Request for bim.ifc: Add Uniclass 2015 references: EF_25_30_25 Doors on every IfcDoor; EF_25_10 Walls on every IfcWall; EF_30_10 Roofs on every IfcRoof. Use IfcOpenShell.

First a look at what the model holds.

```python
import ifcopenshell

model = ifcopenshell.open("bim.ifc")
print(model.schema)
print("classifications:", [c.Name for c in model.by_type("IfcClassification")])
for ifc_class in ("IfcDoor", "IfcRoof", "IfcStair", "IfcWall", "IfcWindow"):
    print(ifc_class, len(model.by_type(ifc_class)))
```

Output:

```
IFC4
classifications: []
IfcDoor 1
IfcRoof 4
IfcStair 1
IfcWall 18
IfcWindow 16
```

```python
import ifcopenshell
import ifcopenshell.api.classification

model = ifcopenshell.open("bim.ifc")

system = ifcopenshell.api.classification.add_classification(model, classification="Uniclass 2015")

codes = {
    "IfcDoor": ("EF_25_30_25", "Doors"),
    "IfcWall": ("EF_25_10", "Walls"),
    "IfcRoof": ("EF_30_10", "Roofs"),
}
for ifc_class, (code, name) in codes.items():
    products = model.by_type(ifc_class)
    ifcopenshell.api.classification.add_reference(
        model, products=products, classification=system, identification=code, name=name
    )
    print(code, len(products))

model.write("bim_updated.ifc")
```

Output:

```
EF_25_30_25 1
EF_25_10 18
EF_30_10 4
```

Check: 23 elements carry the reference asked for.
